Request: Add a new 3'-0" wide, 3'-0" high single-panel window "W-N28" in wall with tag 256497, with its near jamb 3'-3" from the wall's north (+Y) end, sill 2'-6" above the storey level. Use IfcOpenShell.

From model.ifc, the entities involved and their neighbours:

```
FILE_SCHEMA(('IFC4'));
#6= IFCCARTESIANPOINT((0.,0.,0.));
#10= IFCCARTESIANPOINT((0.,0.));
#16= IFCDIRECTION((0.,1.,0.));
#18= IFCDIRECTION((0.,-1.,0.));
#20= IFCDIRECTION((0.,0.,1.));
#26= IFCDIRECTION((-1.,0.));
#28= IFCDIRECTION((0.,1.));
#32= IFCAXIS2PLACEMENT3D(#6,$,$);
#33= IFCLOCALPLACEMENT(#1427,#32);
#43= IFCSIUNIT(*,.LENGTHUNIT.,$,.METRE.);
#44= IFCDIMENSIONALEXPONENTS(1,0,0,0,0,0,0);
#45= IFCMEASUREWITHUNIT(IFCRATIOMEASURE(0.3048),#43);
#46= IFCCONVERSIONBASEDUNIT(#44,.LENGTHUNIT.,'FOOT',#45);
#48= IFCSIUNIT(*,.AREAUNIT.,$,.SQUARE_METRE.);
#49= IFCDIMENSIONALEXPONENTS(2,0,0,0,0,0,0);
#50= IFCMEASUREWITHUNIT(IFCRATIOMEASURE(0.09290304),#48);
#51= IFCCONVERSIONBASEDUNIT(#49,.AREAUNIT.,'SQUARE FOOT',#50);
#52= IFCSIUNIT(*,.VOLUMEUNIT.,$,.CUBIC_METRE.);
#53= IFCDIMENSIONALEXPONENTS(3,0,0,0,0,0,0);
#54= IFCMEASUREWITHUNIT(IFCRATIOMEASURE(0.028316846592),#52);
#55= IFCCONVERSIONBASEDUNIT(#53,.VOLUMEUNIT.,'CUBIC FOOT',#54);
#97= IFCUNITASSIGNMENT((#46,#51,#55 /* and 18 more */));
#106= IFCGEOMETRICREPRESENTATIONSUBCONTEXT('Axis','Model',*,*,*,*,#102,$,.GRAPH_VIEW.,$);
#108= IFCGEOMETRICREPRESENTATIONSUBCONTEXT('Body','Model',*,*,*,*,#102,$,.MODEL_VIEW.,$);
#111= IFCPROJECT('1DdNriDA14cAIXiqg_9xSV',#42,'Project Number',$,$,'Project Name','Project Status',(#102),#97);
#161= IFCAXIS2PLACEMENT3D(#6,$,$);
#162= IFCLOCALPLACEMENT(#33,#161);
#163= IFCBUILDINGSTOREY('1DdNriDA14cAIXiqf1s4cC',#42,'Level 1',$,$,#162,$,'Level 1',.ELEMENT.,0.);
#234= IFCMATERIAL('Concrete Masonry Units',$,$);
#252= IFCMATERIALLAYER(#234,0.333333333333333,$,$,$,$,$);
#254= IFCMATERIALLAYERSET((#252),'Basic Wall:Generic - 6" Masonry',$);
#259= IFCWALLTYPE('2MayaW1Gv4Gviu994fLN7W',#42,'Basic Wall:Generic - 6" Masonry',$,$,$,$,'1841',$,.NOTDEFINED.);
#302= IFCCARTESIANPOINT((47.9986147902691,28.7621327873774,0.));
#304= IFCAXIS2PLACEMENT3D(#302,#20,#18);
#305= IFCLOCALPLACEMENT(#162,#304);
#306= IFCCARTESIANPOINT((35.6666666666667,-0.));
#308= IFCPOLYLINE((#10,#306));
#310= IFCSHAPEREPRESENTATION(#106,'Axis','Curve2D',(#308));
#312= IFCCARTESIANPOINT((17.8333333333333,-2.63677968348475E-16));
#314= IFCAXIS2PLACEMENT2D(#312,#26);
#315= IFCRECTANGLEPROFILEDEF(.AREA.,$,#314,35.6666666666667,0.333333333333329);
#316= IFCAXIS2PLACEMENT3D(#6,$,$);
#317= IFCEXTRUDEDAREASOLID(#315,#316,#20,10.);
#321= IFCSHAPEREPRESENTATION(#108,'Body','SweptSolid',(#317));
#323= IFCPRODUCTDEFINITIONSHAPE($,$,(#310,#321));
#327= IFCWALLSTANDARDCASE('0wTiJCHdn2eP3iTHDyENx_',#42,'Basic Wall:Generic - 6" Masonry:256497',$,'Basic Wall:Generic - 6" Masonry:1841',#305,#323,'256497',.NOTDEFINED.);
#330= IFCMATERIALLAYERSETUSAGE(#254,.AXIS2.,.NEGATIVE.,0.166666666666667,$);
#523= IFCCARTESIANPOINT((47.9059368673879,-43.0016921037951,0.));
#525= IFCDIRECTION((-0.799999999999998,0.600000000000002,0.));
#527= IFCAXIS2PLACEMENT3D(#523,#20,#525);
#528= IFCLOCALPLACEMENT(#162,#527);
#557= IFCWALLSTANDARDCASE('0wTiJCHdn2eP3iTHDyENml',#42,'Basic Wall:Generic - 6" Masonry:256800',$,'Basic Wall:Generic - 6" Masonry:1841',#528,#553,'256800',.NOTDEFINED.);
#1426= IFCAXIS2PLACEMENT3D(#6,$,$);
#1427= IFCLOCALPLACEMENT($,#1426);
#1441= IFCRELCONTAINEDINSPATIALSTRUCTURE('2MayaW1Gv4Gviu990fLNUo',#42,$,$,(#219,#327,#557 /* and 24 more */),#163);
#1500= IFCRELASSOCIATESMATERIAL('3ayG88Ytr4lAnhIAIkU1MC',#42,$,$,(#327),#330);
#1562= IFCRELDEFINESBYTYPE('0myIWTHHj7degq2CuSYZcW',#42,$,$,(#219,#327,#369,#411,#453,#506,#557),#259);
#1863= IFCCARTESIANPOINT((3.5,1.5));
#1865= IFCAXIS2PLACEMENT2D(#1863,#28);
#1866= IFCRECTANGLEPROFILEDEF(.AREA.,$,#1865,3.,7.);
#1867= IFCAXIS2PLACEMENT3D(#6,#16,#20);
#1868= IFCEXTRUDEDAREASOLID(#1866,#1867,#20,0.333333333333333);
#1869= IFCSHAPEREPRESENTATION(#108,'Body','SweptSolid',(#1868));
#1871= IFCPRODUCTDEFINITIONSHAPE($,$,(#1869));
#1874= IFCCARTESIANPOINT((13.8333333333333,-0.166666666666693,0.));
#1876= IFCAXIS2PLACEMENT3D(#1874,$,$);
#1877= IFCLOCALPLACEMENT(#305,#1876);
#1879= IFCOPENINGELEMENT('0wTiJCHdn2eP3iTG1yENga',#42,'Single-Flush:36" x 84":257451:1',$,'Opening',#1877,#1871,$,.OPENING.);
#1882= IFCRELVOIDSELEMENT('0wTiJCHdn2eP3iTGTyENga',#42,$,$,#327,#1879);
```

```python
import numpy as np
import ifcopenshell
import ifcopenshell.api.feature
import ifcopenshell.api.geometry
import ifcopenshell.api.root
import ifcopenshell.api.spatial
import ifcopenshell.geom
import ifcopenshell.util.element
import ifcopenshell.util.placement
import ifcopenshell.util.representation
import ifcopenshell.util.shape
import ifcopenshell.util.unit

model = ifcopenshell.open("model.ifc")
unit_scale = ifcopenshell.util.unit.calculate_unit_scale(model)
settings = ifcopenshell.geom.settings()


def volume(element):
    """Net volume in cubic metres, openings subtracted."""
    shape = ifcopenshell.geom.create_shape(settings, element)
    return ifcopenshell.util.shape.get_volume(shape.geometry)


wall = model.by_id(327)
storey = ifcopenshell.util.element.get_container(wall, ifc_class="IfcBuildingStorey")
context = ifcopenshell.util.representation.get_context(model, "Model", "Body", "MODEL_VIEW")
before = volume(wall)

width, height, from_end, sill = 0.9144, 0.9144, 0.9906, 0.762  # metres

# The wall runs along its own X axis, and the end named is its -X end.
wall_shape = ifcopenshell.geom.create_shape(settings, wall)
x, y, z = ifcopenshell.util.shape.get_vertices(wall_shape.geometry).T
start = x.min() + from_end
face, thickness = float(y.min()), float(y.max() - y.min())
wall_matrix = ifcopenshell.util.placement.get_local_placement(wall.ObjectPlacement)
level = ifcopenshell.util.placement.get_local_placement(storey.ObjectPlacement)[2, 3]


def in_wall(x, y):
    """Placement at x, y metres in the wall's axes, at sill height."""
    matrix = wall_matrix.copy()
    matrix[:, 3] = wall_matrix @ np.array([x / unit_scale, y / unit_scale, 0.0, 1.0])
    matrix[2, 3] = level + sill / unit_scale
    return matrix


# Opening: a box that overshoots both wall faces by 50 mm.
opening = ifcopenshell.api.root.create_entity(model, ifc_class="IfcOpeningElement", predefined_type="OPENING")
box = ifcopenshell.api.geometry.add_wall_representation(
    model, context=context, length=width, height=height, thickness=thickness + 0.1
)
ifcopenshell.api.geometry.assign_representation(model, product=opening, representation=box)
ifcopenshell.api.geometry.edit_object_placement(model, product=opening, matrix=in_wall(start, face - 0.05), is_si=False)
ifcopenshell.api.feature.add_feature(model, feature=opening, element=wall)

window = ifcopenshell.api.root.create_entity(model, ifc_class="IfcWindow", name="W-N28", predefined_type="WINDOW")
window.OverallWidth, window.OverallHeight = width / unit_scale, height / unit_scale
window.PartitioningType = "SINGLE_PANEL"
body = ifcopenshell.api.geometry.add_window_representation(
    model,
    context=context,
    overall_width=window.OverallWidth,
    overall_height=window.OverallHeight,
    partition_type="SINGLE_PANEL",
)
ifcopenshell.api.geometry.assign_representation(model, product=window, representation=body)
ifcopenshell.api.spatial.assign_container(model, products=[window], relating_structure=storey)
ifcopenshell.api.feature.add_filling(model, opening=opening, element=window)

# Centre the window in the wall's thickness.
ifcopenshell.api.geometry.edit_object_placement(model, product=window, matrix=in_wall(start, face), is_si=False)
window_shape = ifcopenshell.geom.create_shape(settings, window)
depth = ifcopenshell.util.shape.get_vertices(window_shape.geometry)[:, 1]
offset = face + thickness / 2 - (depth.min() + depth.max()) / 2
ifcopenshell.api.geometry.edit_object_placement(model, product=window, matrix=in_wall(start, offset), is_si=False)

after = volume(wall)

print(f"wall volume {before:.3f} -> {after:.3f} m3")

model.write("model_v2.ifc")
```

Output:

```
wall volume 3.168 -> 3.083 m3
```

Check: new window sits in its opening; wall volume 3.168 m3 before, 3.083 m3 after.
